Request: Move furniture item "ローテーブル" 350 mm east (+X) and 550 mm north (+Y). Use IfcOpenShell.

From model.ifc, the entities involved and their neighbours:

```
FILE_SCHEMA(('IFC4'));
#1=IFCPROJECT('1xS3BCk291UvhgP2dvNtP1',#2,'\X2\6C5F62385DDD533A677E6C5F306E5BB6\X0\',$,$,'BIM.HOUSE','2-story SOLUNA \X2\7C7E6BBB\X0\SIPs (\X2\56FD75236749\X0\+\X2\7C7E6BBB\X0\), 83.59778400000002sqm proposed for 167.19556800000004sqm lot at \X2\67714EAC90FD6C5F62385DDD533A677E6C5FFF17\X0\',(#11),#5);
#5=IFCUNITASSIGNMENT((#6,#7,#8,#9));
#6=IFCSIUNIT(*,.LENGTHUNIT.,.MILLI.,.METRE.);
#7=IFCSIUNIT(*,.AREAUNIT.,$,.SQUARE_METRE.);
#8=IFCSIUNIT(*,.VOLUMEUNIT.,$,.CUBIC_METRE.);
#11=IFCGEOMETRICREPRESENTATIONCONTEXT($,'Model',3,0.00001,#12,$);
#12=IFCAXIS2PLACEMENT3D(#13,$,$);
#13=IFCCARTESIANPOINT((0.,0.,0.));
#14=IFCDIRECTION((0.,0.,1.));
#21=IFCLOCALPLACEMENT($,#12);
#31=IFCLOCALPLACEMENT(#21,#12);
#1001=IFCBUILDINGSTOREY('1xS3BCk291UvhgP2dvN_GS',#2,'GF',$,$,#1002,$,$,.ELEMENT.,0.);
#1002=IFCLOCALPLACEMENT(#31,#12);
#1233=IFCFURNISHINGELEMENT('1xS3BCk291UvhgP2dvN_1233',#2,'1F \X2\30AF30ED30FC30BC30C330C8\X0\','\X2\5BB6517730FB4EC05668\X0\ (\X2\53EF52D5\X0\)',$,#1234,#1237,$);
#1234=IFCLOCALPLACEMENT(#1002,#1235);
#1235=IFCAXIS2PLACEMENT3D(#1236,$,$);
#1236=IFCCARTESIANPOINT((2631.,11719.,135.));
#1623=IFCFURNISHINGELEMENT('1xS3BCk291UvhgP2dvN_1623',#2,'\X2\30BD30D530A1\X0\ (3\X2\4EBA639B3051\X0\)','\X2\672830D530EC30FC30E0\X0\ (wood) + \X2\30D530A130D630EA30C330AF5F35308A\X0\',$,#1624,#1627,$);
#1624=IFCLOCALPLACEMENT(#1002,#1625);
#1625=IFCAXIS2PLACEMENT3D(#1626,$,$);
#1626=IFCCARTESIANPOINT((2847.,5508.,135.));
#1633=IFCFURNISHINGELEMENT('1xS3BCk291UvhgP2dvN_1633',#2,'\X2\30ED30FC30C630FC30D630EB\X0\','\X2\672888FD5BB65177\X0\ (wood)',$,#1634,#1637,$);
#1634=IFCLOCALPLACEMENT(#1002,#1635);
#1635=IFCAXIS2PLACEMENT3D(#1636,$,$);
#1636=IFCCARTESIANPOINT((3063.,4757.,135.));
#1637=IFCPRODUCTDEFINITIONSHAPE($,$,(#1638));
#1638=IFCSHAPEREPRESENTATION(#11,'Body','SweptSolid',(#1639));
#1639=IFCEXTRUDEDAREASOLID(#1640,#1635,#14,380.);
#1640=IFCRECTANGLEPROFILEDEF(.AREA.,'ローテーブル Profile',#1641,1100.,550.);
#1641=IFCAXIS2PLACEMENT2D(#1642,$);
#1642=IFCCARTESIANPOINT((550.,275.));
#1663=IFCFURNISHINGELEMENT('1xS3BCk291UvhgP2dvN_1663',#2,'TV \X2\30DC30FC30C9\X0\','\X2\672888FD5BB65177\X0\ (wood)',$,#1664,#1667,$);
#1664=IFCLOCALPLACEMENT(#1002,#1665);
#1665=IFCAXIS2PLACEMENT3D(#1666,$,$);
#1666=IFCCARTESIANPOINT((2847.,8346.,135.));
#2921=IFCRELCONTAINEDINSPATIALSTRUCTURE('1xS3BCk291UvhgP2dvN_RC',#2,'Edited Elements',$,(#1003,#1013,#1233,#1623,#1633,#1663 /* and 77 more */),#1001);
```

```python
import ifcopenshell
import ifcopenshell.api.geometry
import ifcopenshell.util.placement
import ifcopenshell.util.unit

model = ifcopenshell.open("model.ifc")
unit_scale = ifcopenshell.util.unit.calculate_unit_scale(model)

item = model.by_guid("1xS3BCk291UvhgP2dvN_1633")
matrix = ifcopenshell.util.placement.get_local_placement(item.ObjectPlacement)
matrix[0, 3] += 0.35 / unit_scale
matrix[1, 3] += 0.55 / unit_scale
ifcopenshell.api.geometry.edit_object_placement(model, product=item, matrix=matrix, is_si=False)

print(ifcopenshell.util.placement.get_local_placement(item.ObjectPlacement).round(3) + 0.0)

model.write("model_rev.ifc")
```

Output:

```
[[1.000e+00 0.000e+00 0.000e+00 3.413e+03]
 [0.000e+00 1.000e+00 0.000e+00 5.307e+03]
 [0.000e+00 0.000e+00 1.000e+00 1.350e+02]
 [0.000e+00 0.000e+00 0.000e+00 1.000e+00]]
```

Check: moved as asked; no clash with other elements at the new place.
